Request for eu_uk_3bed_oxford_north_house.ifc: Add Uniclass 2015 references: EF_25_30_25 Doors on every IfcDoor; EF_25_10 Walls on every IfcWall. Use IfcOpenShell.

First a look at what the model holds.

```python
import ifcopenshell

model = ifcopenshell.open("eu_uk_3bed_oxford_north_house.ifc")
print(model.schema)
print("classifications:", [c.Name for c in model.by_type("IfcClassification")])
for ifc_class in ("IfcDoor", "IfcRoof", "IfcStair", "IfcWall", "IfcWindow"):
    print(ifc_class, len(model.by_type(ifc_class)))
```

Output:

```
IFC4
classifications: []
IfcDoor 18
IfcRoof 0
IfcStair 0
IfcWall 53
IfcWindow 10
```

```python
import ifcopenshell
import ifcopenshell.api.classification

model = ifcopenshell.open("eu_uk_3bed_oxford_north_house.ifc")

system = ifcopenshell.api.classification.add_classification(model, classification="Uniclass 2015")

codes = {
    "IfcDoor": ("EF_25_30_25", "Doors"),
    "IfcWall": ("EF_25_10", "Walls"),
}
for ifc_class, (code, name) in codes.items():
    products = model.by_type(ifc_class)
    ifcopenshell.api.classification.add_reference(
        model, products=products, classification=system, identification=code, name=name
    )
    print(code, len(products))

model.write("eu_uk_3bed_oxford_north_house-out.ifc")
```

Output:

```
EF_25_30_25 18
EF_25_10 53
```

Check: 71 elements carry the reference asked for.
